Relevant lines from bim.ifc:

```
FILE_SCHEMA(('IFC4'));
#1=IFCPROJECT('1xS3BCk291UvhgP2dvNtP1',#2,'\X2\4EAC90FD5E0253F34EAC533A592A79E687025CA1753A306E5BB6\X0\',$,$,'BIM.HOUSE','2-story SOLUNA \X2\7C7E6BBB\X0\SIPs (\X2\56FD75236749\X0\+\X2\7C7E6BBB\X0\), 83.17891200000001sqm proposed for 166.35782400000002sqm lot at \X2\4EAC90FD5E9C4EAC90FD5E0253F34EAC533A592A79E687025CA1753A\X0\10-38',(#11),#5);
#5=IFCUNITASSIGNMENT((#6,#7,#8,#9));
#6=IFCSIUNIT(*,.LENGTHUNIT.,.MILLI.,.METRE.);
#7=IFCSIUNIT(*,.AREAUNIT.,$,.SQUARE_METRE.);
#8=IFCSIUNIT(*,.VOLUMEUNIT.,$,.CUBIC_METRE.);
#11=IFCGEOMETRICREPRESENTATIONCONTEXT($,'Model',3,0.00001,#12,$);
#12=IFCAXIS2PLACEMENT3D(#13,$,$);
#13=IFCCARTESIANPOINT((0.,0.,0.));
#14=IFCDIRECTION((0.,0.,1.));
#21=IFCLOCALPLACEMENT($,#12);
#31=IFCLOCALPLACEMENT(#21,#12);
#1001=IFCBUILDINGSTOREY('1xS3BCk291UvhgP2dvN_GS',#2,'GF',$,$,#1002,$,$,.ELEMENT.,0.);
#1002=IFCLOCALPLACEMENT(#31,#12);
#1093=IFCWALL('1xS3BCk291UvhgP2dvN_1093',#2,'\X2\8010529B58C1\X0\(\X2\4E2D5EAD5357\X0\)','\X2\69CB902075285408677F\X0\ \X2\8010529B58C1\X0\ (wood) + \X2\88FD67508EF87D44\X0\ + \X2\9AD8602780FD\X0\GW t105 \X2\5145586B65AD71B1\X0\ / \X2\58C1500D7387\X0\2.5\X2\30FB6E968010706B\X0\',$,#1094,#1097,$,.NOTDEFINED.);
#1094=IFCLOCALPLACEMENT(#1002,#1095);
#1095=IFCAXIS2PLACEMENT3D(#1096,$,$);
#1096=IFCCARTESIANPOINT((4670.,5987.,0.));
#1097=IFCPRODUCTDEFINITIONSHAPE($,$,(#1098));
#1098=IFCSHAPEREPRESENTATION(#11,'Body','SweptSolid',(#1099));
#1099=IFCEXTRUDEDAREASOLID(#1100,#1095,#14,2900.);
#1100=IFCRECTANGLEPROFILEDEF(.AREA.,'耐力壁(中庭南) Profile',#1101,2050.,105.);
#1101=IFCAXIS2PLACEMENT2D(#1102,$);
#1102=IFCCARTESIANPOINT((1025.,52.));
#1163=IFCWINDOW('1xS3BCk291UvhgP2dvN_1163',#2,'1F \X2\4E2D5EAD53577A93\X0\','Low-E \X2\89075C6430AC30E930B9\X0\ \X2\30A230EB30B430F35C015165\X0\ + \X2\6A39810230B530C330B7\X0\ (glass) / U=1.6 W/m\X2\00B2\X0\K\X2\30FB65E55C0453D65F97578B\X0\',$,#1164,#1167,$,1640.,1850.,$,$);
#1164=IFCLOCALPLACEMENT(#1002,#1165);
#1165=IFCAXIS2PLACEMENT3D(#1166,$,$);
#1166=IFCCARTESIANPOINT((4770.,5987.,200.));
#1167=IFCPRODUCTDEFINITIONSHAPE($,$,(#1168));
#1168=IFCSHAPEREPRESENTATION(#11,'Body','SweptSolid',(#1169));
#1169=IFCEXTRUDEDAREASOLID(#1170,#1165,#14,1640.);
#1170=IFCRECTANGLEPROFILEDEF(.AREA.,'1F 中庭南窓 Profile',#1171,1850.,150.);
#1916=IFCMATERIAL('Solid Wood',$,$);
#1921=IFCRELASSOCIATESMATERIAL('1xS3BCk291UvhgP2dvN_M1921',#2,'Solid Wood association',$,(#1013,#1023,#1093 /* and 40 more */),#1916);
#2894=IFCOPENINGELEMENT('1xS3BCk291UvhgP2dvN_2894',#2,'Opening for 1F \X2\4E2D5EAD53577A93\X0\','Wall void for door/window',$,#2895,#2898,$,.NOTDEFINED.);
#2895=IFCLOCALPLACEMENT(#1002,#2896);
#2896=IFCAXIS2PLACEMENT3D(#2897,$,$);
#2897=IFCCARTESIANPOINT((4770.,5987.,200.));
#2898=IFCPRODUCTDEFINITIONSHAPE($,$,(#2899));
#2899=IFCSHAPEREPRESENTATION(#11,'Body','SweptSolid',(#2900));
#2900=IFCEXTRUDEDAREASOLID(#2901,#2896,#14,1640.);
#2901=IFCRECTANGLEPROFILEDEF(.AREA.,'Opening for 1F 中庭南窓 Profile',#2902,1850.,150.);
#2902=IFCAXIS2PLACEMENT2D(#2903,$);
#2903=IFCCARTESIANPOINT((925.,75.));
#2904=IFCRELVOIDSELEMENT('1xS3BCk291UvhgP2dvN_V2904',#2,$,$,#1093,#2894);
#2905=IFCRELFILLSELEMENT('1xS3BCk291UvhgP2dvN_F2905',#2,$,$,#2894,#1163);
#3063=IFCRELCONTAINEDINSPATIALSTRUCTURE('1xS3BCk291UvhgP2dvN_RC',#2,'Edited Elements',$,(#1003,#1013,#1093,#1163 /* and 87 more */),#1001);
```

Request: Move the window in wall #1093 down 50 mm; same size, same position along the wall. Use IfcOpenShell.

```python
import numpy as np
import ifcopenshell
import ifcopenshell.api.geometry
import ifcopenshell.util.placement
import ifcopenshell.util.unit

model = ifcopenshell.open("bim.ifc")
unit_scale = ifcopenshell.util.unit.calculate_unit_scale(model)

window = model.by_guid("1xS3BCk291UvhgP2dvN_1163")
opening = window.FillsVoids[0].RelatingOpeningElement
dz = -50.0

shift = np.array([0.0, 0.0, dz])
# The window is not placed relative to its opening, so move both.
for product in (opening, window):
    matrix = ifcopenshell.util.placement.get_local_placement(product.ObjectPlacement)
    matrix[:3, 3] += shift
    ifcopenshell.api.geometry.edit_object_placement(model, product=product, matrix=matrix, is_si=False)

print(f"moved by {dz * unit_scale:+.3f} m")

model.write("bim_edited.ifc")
```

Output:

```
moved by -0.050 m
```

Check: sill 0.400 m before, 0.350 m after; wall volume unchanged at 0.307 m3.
